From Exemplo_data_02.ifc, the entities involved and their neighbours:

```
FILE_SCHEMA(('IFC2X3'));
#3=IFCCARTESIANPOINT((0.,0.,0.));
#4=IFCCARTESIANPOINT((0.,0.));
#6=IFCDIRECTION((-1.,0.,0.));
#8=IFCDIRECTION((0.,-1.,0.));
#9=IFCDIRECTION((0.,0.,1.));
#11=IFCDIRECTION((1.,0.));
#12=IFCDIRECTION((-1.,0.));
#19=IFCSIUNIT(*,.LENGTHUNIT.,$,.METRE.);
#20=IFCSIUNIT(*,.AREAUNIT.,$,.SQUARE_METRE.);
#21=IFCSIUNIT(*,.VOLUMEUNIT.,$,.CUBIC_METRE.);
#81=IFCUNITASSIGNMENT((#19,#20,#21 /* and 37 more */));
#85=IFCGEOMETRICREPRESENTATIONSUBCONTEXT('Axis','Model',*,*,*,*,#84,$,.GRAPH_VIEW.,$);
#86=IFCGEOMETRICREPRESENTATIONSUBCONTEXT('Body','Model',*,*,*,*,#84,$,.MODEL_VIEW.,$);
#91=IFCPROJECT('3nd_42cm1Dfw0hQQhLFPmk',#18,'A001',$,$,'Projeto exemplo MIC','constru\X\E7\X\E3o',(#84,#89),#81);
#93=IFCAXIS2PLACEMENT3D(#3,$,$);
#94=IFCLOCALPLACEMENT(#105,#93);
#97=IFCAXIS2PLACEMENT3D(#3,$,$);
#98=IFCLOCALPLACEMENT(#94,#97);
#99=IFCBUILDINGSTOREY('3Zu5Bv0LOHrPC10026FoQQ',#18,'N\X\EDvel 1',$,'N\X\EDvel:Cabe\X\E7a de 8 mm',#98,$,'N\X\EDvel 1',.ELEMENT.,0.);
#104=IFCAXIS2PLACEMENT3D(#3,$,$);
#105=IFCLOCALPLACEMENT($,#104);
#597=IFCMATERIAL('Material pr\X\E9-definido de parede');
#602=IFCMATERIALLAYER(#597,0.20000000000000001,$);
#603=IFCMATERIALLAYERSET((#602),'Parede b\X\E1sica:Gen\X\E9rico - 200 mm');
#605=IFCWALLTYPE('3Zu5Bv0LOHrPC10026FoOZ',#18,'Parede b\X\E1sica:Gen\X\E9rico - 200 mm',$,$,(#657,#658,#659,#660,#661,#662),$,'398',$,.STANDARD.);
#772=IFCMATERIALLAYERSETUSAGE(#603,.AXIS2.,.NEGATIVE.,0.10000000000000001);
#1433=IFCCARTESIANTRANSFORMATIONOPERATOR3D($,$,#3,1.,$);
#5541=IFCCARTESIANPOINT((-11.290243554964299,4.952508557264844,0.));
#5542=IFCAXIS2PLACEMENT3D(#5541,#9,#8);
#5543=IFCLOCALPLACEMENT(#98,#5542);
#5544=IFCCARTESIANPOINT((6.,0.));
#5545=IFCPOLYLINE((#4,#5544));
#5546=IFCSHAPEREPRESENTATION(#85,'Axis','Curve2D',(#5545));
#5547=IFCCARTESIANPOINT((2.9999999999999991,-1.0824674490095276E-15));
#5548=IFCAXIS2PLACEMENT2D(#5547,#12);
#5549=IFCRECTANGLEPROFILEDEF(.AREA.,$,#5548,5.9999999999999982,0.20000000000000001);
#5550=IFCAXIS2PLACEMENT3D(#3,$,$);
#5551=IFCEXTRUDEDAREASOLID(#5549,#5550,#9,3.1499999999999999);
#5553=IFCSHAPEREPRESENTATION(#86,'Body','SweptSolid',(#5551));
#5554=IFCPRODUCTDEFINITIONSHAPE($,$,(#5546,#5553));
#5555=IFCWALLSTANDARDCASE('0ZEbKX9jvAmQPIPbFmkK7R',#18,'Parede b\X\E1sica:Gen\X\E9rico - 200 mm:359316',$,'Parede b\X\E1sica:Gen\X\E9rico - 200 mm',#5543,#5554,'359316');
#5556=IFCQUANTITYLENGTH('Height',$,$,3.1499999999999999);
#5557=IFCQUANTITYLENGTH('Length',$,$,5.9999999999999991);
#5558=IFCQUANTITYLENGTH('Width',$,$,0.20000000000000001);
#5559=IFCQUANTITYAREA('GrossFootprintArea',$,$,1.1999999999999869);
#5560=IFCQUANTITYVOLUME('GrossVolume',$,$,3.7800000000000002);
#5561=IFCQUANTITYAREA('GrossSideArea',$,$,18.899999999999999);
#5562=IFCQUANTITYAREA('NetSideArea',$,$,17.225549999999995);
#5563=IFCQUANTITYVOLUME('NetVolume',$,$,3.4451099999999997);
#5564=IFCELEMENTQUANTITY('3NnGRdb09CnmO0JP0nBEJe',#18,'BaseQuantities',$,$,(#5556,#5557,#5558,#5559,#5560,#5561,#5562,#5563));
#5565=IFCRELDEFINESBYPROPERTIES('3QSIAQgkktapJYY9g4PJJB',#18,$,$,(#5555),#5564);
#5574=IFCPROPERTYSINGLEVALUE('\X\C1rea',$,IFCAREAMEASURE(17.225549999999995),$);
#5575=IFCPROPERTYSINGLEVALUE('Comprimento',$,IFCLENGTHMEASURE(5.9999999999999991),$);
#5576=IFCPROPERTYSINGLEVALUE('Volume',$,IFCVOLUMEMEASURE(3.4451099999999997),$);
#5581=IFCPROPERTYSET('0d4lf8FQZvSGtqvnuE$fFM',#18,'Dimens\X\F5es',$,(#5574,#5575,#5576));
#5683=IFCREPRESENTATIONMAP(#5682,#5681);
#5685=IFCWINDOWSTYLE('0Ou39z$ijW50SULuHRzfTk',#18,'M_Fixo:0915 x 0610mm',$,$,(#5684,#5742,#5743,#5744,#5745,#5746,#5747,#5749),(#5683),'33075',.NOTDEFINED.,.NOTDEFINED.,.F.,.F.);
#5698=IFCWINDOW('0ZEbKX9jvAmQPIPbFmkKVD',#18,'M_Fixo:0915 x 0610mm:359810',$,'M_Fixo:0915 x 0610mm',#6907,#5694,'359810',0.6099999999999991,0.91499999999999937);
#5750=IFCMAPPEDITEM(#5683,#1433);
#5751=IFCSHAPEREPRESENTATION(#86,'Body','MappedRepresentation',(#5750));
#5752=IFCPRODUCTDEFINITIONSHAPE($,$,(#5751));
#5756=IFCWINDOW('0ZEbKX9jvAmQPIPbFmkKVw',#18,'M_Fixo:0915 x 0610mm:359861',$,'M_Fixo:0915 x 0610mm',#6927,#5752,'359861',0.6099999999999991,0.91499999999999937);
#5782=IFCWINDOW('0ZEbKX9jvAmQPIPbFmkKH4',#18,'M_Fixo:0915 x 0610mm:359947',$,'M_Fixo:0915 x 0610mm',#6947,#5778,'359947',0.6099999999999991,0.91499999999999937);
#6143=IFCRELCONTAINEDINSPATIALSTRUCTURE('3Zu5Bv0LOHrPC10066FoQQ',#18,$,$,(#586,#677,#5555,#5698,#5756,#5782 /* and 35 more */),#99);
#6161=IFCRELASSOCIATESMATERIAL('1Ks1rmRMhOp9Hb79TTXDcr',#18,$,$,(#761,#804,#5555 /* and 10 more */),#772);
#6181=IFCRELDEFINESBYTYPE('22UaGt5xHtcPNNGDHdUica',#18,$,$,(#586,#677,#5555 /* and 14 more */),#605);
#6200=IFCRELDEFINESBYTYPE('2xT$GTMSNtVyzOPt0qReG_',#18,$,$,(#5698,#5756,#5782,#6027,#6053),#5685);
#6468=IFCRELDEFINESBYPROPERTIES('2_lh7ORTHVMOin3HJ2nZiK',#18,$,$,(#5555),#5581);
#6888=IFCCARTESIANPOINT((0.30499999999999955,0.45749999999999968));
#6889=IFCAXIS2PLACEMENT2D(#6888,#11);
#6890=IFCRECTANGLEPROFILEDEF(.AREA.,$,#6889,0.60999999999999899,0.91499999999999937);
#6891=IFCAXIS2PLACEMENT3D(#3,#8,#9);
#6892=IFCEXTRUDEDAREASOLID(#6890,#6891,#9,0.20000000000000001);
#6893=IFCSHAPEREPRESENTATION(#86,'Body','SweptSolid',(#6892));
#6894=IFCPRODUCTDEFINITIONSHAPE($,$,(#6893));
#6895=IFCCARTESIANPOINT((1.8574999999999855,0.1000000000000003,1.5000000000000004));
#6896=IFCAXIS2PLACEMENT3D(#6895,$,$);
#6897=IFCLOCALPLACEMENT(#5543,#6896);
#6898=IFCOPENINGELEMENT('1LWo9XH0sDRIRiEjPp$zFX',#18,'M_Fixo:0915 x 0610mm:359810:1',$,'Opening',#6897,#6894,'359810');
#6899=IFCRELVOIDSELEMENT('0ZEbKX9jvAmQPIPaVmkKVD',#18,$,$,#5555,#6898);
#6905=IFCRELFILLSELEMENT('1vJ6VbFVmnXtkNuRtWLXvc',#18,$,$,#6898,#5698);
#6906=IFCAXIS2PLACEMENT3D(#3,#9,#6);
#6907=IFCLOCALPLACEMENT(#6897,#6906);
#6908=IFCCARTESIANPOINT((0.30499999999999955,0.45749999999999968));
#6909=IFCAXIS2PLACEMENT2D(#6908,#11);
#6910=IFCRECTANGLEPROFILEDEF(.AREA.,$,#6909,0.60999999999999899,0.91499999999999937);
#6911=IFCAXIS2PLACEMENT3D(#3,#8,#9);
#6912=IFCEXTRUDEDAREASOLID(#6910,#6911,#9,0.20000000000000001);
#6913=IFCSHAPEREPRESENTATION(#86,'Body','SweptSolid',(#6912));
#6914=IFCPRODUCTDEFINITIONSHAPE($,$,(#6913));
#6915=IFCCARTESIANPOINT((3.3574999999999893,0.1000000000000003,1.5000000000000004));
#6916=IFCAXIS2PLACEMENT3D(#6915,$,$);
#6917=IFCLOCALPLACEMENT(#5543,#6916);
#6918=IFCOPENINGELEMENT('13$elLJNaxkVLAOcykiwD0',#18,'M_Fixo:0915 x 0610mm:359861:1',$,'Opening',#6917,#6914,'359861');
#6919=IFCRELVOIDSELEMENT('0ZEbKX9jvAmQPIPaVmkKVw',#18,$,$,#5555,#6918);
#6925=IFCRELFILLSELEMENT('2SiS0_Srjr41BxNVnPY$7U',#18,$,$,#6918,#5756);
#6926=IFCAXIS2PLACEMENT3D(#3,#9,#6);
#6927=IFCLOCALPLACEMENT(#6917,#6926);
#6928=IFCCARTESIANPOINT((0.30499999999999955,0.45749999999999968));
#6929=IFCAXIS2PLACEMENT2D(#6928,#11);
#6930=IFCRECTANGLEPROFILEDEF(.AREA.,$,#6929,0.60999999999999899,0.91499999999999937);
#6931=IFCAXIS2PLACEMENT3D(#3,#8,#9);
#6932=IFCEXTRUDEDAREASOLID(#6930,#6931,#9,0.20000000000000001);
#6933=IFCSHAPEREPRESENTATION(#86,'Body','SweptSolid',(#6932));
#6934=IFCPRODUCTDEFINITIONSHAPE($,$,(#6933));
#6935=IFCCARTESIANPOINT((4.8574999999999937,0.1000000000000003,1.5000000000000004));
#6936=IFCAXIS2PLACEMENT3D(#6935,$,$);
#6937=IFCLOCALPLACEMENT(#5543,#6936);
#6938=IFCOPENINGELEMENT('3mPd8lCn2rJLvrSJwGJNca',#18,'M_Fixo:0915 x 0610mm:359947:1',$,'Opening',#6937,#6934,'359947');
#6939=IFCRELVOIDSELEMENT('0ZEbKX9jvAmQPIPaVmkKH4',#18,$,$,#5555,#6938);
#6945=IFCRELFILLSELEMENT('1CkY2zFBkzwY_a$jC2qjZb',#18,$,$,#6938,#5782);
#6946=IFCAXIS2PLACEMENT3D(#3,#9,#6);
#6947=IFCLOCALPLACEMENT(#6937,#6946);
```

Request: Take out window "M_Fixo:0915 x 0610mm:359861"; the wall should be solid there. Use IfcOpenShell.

```python
import ifcopenshell
import ifcopenshell.api.feature
import ifcopenshell.api.pset
import ifcopenshell.api.root
import ifcopenshell.geom
import ifcopenshell.util.element
import ifcopenshell.util.shape
import ifcopenshell.util.unit

model = ifcopenshell.open("Exemplo_data_02.ifc")
area_scale = ifcopenshell.util.unit.calculate_unit_scale(model, "AREAUNIT")
volume_scale = ifcopenshell.util.unit.calculate_unit_scale(model, "VOLUMEUNIT")
settings = ifcopenshell.geom.settings()


def volume(element):
    """Net volume in cubic metres, openings subtracted."""
    shape = ifcopenshell.geom.create_shape(settings, element)
    return ifcopenshell.util.shape.get_volume(shape.geometry)


window = model.by_guid("0ZEbKX9jvAmQPIPbFmkKVw")
opening = window.FillsVoids[0].RelatingOpeningElement
wall = opening.VoidsElements[0].RelatingBuildingElement
before = volume(wall)

ifcopenshell.api.root.remove_product(model, product=window)
ifcopenshell.api.feature.remove_feature(model, feature=opening)

after = volume(wall)
thickness = 0.2  # wall thickness in metres

# Update the wall's stored quantities.
qto = model.by_id(ifcopenshell.util.element.get_pset(wall, "BaseQuantities", should_inherit=False)["id"])
ifcopenshell.api.pset.edit_qto(model, qto=qto, properties={
    "NetSideArea": after / thickness / area_scale,
    "NetVolume": after / volume_scale,
})
pset = model.by_id(ifcopenshell.util.element.get_pset(wall, "Dimensões", should_inherit=False)["id"])
ifcopenshell.api.pset.edit_pset(model, pset=pset, properties={
    "Área": model.create_entity("IfcAreaMeasure", after / thickness / area_scale),
    "Volume": model.create_entity("IfcVolumeMeasure", after / volume_scale),
})

print(f"wall volume {before:.3f} -> {after:.3f} m3")

model.write("Exemplo_data_02-out.ifc")
```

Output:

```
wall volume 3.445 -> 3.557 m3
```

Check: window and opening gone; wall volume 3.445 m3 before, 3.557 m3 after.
